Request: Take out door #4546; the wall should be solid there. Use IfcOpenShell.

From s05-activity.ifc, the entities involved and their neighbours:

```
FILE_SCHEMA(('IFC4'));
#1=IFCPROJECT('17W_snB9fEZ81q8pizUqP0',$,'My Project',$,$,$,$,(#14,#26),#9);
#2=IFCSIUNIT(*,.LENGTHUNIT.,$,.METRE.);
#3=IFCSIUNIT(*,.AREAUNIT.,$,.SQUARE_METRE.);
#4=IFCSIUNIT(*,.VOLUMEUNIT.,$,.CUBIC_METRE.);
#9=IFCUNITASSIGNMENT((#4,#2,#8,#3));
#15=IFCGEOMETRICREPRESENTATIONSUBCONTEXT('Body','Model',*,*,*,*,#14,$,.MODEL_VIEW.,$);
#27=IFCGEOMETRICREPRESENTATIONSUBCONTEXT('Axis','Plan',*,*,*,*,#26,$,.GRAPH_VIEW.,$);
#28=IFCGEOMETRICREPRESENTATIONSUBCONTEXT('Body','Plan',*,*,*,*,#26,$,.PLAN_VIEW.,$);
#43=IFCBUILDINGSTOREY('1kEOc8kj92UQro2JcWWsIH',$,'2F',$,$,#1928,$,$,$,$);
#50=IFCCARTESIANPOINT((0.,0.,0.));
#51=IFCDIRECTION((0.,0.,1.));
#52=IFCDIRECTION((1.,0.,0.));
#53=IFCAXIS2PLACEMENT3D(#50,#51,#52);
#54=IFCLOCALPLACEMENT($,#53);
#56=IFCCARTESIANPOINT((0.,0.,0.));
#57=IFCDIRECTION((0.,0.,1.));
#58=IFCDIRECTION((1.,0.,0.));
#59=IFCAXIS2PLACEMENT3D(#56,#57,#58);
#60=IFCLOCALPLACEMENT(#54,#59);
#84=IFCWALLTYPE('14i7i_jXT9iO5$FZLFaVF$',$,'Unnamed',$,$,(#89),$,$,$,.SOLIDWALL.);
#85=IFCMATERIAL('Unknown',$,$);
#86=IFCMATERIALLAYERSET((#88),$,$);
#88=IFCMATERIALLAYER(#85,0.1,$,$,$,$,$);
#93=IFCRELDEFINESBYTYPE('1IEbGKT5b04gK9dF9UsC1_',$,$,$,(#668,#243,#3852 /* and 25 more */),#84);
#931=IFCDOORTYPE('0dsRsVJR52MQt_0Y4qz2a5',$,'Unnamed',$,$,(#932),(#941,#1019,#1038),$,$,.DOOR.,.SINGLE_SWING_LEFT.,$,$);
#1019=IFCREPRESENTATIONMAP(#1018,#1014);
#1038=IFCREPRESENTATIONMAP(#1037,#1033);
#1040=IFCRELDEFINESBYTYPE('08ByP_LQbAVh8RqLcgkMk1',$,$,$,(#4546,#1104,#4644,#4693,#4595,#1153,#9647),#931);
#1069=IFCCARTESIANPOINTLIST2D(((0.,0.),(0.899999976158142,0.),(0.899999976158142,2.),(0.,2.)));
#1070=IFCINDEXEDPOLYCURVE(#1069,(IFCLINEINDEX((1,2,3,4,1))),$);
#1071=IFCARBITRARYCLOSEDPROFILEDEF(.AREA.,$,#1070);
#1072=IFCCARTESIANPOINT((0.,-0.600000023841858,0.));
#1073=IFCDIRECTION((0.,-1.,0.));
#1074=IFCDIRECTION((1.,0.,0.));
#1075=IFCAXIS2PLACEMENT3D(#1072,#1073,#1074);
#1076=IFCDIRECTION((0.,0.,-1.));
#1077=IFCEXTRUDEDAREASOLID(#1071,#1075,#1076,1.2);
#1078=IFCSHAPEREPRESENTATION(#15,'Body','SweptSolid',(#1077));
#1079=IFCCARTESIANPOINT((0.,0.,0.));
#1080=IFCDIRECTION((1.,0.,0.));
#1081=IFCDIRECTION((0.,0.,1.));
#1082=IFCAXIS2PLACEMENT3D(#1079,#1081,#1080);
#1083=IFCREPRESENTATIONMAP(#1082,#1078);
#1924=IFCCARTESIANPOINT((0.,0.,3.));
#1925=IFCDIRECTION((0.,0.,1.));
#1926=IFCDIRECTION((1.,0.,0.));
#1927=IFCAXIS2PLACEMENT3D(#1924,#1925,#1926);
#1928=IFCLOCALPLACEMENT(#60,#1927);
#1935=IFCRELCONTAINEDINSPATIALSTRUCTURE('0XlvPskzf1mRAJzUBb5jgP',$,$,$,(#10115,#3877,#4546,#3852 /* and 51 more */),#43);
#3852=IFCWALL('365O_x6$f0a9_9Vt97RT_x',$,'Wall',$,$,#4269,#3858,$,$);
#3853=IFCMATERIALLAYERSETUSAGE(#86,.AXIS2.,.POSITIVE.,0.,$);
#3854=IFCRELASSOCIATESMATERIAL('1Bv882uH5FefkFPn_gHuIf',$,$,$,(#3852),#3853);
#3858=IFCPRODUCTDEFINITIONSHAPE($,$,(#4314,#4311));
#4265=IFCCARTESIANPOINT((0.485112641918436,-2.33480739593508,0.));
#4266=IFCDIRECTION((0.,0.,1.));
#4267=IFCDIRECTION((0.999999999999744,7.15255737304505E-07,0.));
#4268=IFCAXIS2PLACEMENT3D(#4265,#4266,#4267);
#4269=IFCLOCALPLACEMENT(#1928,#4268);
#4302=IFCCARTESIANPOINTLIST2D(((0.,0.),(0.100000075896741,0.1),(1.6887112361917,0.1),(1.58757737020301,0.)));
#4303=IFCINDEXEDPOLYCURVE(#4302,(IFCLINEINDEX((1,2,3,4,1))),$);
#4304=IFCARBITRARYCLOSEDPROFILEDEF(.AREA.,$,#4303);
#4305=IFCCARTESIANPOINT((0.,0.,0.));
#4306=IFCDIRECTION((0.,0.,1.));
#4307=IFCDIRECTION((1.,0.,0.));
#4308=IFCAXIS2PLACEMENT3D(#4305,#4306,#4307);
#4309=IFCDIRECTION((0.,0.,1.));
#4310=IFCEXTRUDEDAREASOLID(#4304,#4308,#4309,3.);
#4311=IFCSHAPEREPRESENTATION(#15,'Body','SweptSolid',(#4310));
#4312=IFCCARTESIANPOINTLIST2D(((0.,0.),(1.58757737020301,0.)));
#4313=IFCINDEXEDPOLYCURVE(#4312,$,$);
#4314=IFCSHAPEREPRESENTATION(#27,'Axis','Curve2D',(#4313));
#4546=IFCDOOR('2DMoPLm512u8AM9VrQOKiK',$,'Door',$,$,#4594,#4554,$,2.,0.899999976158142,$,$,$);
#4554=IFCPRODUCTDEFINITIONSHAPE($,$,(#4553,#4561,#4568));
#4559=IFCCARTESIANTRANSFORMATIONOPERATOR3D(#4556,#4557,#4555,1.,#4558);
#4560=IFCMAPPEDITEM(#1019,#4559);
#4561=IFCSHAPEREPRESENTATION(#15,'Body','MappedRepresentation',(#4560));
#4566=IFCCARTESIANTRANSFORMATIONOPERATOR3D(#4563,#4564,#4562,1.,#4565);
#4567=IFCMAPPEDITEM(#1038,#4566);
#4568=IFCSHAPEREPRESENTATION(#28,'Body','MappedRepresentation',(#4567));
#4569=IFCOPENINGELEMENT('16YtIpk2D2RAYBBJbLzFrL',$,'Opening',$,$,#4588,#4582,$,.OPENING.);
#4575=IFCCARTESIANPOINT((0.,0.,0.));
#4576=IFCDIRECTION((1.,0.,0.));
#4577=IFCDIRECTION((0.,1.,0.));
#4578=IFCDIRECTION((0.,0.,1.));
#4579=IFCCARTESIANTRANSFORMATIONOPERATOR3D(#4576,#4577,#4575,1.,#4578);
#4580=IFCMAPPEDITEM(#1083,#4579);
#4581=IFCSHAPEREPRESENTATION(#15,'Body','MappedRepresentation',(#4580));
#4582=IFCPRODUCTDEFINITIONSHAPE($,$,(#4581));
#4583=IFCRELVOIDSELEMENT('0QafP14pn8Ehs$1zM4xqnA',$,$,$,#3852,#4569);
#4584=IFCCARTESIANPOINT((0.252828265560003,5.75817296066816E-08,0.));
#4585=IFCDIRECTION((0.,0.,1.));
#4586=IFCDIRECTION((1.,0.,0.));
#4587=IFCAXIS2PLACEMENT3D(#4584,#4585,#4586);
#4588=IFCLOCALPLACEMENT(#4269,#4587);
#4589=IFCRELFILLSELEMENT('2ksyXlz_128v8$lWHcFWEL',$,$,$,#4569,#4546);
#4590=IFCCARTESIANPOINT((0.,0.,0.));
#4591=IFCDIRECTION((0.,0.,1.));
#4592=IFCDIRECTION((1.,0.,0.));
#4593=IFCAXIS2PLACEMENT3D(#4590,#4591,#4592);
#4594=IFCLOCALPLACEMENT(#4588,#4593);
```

```python
import ifcopenshell
import ifcopenshell.api.feature
import ifcopenshell.api.root
import ifcopenshell.geom
import ifcopenshell.util.shape

model = ifcopenshell.open("s05-activity.ifc")
settings = ifcopenshell.geom.settings()


def volume(element):
    """Net volume in cubic metres, openings subtracted."""
    shape = ifcopenshell.geom.create_shape(settings, element)
    return ifcopenshell.util.shape.get_volume(shape.geometry)


door = model.by_guid("2DMoPLm512u8AM9VrQOKiK")
opening = door.FillsVoids[0].RelatingOpeningElement
wall = opening.VoidsElements[0].RelatingBuildingElement
before = volume(wall)

ifcopenshell.api.root.remove_product(model, product=door)
ifcopenshell.api.feature.remove_feature(model, feature=opening)

after = volume(wall)

print(f"wall volume {before:.3f} -> {after:.3f} m3")

model.write("s05-activity_v2.ifc")
```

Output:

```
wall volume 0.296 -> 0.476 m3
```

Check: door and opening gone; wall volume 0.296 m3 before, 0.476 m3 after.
